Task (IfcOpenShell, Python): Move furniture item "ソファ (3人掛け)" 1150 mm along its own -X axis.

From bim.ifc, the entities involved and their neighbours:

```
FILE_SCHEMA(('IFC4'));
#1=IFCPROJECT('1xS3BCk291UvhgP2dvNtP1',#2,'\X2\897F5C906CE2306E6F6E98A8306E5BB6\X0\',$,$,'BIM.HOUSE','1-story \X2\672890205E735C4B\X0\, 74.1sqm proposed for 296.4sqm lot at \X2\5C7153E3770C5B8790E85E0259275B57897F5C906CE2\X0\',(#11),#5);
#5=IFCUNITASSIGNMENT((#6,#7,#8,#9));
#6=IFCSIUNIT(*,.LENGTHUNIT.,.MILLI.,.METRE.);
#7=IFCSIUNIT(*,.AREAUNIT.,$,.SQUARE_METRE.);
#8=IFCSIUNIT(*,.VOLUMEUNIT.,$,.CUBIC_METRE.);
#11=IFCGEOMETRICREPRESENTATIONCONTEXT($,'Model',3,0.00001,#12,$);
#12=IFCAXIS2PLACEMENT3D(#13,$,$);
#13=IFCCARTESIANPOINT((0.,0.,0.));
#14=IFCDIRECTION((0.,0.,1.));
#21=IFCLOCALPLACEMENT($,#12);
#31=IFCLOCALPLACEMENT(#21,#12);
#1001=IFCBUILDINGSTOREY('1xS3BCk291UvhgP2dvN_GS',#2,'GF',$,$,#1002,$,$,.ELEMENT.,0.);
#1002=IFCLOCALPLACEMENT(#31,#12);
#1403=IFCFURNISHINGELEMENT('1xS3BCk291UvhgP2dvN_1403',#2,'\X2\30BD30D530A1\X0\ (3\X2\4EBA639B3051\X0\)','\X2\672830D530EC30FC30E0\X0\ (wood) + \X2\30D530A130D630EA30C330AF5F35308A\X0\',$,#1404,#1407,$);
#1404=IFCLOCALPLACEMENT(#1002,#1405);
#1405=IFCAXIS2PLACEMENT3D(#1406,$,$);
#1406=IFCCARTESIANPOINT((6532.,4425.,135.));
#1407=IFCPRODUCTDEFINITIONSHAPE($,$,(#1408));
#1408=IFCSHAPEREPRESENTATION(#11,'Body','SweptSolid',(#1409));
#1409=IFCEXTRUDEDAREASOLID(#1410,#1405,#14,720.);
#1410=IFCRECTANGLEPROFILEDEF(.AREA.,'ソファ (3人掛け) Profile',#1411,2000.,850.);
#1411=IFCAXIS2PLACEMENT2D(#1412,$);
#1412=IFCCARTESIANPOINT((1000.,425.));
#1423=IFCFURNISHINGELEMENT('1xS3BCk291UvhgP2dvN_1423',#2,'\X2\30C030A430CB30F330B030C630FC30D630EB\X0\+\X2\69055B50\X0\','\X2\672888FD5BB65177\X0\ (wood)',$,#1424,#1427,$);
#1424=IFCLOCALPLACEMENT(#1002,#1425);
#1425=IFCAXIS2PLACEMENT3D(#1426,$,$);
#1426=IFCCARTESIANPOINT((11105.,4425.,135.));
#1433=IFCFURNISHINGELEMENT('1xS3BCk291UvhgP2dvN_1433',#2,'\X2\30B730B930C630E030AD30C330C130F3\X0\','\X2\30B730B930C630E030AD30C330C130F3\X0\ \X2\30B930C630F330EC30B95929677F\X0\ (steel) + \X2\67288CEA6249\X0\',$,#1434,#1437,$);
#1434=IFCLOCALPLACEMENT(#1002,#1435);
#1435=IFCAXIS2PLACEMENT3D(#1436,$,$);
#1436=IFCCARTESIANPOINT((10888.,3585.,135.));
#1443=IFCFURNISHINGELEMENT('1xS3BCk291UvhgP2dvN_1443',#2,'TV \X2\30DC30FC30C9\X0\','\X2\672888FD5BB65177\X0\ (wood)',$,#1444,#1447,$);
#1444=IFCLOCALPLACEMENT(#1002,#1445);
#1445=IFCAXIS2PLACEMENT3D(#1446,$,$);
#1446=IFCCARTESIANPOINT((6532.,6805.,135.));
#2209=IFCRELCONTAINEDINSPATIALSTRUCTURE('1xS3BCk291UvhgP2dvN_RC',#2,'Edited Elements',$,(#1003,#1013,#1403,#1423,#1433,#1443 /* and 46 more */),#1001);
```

```python
import ifcopenshell
import ifcopenshell.api.geometry
import ifcopenshell.util.placement
import ifcopenshell.util.unit

model = ifcopenshell.open("bim.ifc")
unit_scale = ifcopenshell.util.unit.calculate_unit_scale(model)

item = model.by_guid("1xS3BCk291UvhgP2dvN_1403")
matrix = ifcopenshell.util.placement.get_local_placement(item.ObjectPlacement)
matrix[:3, 3] -= matrix[:3, 0] * 1.15 / unit_scale
ifcopenshell.api.geometry.edit_object_placement(model, product=item, matrix=matrix, is_si=False)

print(ifcopenshell.util.placement.get_local_placement(item.ObjectPlacement).round(3) + 0.0)

model.write("bim_edited.ifc")
```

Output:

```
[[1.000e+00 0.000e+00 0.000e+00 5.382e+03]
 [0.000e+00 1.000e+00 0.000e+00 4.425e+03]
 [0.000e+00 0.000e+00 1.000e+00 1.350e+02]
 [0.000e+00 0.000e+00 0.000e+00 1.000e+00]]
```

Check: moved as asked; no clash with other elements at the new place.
